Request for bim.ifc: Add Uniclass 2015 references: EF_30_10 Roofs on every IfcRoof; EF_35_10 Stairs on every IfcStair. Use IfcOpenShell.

First a look at what the model holds.

```python
import ifcopenshell

model = ifcopenshell.open("bim.ifc")
print(model.schema)
print("classifications:", [c.Name for c in model.by_type("IfcClassification")])
for ifc_class in ("IfcDoor", "IfcRoof", "IfcStair", "IfcWall", "IfcWindow"):
    print(ifc_class, len(model.by_type(ifc_class)))
```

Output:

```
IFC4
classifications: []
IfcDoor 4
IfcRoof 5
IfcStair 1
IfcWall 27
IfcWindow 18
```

```python
import ifcopenshell
import ifcopenshell.api.classification

model = ifcopenshell.open("bim.ifc")

system = ifcopenshell.api.classification.add_classification(model, classification="Uniclass 2015")

codes = {
    "IfcRoof": ("EF_30_10", "Roofs"),
    "IfcStair": ("EF_35_10", "Stairs"),
}
for ifc_class, (code, name) in codes.items():
    products = model.by_type(ifc_class)
    ifcopenshell.api.classification.add_reference(
        model, products=products, classification=system, identification=code, name=name
    )
    print(code, len(products))

model.write("bim-out.ifc")
```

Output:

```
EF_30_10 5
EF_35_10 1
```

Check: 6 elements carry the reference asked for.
